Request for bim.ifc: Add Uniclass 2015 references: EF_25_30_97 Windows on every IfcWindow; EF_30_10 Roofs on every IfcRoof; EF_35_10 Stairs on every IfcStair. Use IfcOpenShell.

First a look at what the model holds.

```python
import ifcopenshell

model = ifcopenshell.open("bim.ifc")
print(model.schema)
print("classifications:", [c.Name for c in model.by_type("IfcClassification")])
for ifc_class in ("IfcDoor", "IfcRoof", "IfcStair", "IfcWall", "IfcWindow"):
    print(ifc_class, len(model.by_type(ifc_class)))
```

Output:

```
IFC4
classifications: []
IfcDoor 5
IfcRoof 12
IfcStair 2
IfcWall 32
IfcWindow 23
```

```python
import ifcopenshell
import ifcopenshell.api.classification

model = ifcopenshell.open("bim.ifc")

system = ifcopenshell.api.classification.add_classification(model, classification="Uniclass 2015")

codes = {
    "IfcWindow": ("EF_25_30_97", "Windows"),
    "IfcRoof": ("EF_30_10", "Roofs"),
    "IfcStair": ("EF_35_10", "Stairs"),
}
for ifc_class, (code, name) in codes.items():
    products = model.by_type(ifc_class)
    ifcopenshell.api.classification.add_reference(
        model, products=products, classification=system, identification=code, name=name
    )
    print(code, len(products))

model.write("bim_v2.ifc")
```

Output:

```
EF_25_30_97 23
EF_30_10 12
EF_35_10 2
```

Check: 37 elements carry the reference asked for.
